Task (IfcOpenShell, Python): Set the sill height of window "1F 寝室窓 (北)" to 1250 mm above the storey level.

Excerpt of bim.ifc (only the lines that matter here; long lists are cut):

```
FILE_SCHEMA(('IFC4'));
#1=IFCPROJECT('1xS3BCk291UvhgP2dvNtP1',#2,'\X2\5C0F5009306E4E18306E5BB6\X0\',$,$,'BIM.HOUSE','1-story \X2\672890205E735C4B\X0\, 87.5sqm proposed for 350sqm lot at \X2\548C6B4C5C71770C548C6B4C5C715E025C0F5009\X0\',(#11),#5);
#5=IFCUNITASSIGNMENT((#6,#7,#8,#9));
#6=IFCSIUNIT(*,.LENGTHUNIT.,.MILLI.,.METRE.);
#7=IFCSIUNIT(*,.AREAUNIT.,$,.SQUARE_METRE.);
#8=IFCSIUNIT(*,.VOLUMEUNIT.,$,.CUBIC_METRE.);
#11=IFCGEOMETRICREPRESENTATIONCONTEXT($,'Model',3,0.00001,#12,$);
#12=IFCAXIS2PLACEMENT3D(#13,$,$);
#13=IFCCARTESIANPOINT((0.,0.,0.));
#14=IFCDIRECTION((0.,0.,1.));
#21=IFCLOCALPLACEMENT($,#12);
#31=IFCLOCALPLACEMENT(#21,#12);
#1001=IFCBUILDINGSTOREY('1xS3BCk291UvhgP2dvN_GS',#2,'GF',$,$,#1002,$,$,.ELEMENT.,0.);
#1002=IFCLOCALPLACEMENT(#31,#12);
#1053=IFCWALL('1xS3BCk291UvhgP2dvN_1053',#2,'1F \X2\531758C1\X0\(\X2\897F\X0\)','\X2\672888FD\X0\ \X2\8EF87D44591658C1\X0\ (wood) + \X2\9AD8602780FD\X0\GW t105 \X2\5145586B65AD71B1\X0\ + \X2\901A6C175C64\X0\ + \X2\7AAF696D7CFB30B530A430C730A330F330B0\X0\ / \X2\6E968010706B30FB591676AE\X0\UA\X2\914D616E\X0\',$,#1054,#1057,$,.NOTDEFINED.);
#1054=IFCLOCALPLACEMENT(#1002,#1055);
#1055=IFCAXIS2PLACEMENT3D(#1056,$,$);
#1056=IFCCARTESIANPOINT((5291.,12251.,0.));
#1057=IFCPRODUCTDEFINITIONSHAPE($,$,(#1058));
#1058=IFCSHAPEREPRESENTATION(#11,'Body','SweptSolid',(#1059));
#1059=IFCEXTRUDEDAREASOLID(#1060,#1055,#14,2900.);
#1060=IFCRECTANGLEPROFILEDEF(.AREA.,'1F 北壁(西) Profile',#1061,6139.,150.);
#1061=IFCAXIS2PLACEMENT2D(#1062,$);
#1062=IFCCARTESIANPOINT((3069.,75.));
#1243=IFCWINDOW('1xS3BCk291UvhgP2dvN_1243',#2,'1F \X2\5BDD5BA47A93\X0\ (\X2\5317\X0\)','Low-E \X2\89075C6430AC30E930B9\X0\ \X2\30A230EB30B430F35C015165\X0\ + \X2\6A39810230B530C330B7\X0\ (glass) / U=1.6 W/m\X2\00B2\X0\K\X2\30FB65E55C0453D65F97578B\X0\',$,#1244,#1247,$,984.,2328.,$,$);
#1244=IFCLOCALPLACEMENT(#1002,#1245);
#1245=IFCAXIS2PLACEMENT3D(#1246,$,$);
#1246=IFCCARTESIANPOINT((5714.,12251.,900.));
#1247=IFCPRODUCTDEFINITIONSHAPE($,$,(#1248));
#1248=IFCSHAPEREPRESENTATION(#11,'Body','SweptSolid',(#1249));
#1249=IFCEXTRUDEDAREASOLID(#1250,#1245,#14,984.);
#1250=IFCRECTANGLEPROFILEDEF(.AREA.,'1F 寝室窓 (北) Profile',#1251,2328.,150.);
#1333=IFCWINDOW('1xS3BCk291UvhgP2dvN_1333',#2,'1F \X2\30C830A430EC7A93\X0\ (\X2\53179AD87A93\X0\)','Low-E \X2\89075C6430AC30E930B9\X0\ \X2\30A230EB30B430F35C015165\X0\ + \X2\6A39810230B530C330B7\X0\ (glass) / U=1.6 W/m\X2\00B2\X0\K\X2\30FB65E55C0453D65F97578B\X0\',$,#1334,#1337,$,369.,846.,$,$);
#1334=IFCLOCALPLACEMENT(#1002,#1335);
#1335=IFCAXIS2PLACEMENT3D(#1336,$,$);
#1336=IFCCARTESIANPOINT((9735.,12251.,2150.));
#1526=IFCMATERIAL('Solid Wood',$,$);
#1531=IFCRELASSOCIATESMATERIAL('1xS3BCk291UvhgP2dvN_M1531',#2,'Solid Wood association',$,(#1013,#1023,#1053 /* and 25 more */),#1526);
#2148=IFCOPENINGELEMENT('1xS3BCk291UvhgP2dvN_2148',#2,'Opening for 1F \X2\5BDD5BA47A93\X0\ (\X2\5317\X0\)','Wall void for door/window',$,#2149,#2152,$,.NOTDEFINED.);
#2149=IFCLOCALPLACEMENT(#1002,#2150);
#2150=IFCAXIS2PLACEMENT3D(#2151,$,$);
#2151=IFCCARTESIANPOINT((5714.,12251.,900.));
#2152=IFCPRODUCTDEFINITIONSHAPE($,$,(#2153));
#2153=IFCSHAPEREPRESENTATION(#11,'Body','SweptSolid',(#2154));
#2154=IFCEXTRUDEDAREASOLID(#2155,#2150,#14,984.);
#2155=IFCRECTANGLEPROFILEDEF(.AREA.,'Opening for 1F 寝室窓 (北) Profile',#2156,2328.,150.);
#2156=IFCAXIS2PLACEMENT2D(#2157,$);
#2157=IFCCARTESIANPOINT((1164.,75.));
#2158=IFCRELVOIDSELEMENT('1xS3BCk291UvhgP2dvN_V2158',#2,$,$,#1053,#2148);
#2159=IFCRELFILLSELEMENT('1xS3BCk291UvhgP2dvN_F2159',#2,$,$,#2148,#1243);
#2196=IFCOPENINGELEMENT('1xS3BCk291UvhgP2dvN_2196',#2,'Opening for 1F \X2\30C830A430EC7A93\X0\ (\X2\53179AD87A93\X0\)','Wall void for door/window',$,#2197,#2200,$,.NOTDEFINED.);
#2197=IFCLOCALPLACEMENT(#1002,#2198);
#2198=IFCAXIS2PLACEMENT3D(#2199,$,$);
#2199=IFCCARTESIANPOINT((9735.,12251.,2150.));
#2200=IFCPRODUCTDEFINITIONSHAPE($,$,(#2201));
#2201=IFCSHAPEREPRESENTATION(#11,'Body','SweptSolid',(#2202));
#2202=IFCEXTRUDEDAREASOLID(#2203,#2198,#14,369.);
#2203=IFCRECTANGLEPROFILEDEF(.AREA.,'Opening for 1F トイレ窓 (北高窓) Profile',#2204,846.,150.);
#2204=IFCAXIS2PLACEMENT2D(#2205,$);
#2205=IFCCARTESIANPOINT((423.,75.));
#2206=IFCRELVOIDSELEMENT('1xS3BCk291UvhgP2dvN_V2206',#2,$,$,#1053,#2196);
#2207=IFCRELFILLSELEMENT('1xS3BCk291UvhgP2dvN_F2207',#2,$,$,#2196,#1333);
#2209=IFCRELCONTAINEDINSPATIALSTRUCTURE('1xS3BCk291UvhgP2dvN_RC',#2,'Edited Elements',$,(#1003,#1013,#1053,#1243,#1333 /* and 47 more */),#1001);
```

```python
import numpy as np
import ifcopenshell
import ifcopenshell.api.geometry
import ifcopenshell.geom
import ifcopenshell.util.element
import ifcopenshell.util.placement
import ifcopenshell.util.shape
import ifcopenshell.util.unit

model = ifcopenshell.open("bim.ifc")
unit_scale = ifcopenshell.util.unit.calculate_unit_scale(model)

window = model.by_guid("1xS3BCk291UvhgP2dvN_1243")
opening = window.FillsVoids[0].RelatingOpeningElement
storey = ifcopenshell.util.element.get_container(window, ifc_class="IfcBuildingStorey")
level = ifcopenshell.util.placement.get_local_placement(storey.ObjectPlacement)[2, 3]

# The opening's origin need not be at the sill, so measure its lowest point.
shape = ifcopenshell.geom.create_shape(ifcopenshell.geom.settings(), opening)
bottom = ifcopenshell.util.shape.get_shape_bottom_elevation(shape, shape.geometry) / unit_scale
dz = level + 1.25 / unit_scale - bottom

shift = np.array([0.0, 0.0, dz])
# The window is not placed relative to its opening, so move both.
for product in (opening, window):
    matrix = ifcopenshell.util.placement.get_local_placement(product.ObjectPlacement)
    matrix[:3, 3] += shift
    ifcopenshell.api.geometry.edit_object_placement(model, product=product, matrix=matrix, is_si=False)

print(f"moved by {dz * unit_scale:+.3f} m")

model.write("bim_v2.ifc")
```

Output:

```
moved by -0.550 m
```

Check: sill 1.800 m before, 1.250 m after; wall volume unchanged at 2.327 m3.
